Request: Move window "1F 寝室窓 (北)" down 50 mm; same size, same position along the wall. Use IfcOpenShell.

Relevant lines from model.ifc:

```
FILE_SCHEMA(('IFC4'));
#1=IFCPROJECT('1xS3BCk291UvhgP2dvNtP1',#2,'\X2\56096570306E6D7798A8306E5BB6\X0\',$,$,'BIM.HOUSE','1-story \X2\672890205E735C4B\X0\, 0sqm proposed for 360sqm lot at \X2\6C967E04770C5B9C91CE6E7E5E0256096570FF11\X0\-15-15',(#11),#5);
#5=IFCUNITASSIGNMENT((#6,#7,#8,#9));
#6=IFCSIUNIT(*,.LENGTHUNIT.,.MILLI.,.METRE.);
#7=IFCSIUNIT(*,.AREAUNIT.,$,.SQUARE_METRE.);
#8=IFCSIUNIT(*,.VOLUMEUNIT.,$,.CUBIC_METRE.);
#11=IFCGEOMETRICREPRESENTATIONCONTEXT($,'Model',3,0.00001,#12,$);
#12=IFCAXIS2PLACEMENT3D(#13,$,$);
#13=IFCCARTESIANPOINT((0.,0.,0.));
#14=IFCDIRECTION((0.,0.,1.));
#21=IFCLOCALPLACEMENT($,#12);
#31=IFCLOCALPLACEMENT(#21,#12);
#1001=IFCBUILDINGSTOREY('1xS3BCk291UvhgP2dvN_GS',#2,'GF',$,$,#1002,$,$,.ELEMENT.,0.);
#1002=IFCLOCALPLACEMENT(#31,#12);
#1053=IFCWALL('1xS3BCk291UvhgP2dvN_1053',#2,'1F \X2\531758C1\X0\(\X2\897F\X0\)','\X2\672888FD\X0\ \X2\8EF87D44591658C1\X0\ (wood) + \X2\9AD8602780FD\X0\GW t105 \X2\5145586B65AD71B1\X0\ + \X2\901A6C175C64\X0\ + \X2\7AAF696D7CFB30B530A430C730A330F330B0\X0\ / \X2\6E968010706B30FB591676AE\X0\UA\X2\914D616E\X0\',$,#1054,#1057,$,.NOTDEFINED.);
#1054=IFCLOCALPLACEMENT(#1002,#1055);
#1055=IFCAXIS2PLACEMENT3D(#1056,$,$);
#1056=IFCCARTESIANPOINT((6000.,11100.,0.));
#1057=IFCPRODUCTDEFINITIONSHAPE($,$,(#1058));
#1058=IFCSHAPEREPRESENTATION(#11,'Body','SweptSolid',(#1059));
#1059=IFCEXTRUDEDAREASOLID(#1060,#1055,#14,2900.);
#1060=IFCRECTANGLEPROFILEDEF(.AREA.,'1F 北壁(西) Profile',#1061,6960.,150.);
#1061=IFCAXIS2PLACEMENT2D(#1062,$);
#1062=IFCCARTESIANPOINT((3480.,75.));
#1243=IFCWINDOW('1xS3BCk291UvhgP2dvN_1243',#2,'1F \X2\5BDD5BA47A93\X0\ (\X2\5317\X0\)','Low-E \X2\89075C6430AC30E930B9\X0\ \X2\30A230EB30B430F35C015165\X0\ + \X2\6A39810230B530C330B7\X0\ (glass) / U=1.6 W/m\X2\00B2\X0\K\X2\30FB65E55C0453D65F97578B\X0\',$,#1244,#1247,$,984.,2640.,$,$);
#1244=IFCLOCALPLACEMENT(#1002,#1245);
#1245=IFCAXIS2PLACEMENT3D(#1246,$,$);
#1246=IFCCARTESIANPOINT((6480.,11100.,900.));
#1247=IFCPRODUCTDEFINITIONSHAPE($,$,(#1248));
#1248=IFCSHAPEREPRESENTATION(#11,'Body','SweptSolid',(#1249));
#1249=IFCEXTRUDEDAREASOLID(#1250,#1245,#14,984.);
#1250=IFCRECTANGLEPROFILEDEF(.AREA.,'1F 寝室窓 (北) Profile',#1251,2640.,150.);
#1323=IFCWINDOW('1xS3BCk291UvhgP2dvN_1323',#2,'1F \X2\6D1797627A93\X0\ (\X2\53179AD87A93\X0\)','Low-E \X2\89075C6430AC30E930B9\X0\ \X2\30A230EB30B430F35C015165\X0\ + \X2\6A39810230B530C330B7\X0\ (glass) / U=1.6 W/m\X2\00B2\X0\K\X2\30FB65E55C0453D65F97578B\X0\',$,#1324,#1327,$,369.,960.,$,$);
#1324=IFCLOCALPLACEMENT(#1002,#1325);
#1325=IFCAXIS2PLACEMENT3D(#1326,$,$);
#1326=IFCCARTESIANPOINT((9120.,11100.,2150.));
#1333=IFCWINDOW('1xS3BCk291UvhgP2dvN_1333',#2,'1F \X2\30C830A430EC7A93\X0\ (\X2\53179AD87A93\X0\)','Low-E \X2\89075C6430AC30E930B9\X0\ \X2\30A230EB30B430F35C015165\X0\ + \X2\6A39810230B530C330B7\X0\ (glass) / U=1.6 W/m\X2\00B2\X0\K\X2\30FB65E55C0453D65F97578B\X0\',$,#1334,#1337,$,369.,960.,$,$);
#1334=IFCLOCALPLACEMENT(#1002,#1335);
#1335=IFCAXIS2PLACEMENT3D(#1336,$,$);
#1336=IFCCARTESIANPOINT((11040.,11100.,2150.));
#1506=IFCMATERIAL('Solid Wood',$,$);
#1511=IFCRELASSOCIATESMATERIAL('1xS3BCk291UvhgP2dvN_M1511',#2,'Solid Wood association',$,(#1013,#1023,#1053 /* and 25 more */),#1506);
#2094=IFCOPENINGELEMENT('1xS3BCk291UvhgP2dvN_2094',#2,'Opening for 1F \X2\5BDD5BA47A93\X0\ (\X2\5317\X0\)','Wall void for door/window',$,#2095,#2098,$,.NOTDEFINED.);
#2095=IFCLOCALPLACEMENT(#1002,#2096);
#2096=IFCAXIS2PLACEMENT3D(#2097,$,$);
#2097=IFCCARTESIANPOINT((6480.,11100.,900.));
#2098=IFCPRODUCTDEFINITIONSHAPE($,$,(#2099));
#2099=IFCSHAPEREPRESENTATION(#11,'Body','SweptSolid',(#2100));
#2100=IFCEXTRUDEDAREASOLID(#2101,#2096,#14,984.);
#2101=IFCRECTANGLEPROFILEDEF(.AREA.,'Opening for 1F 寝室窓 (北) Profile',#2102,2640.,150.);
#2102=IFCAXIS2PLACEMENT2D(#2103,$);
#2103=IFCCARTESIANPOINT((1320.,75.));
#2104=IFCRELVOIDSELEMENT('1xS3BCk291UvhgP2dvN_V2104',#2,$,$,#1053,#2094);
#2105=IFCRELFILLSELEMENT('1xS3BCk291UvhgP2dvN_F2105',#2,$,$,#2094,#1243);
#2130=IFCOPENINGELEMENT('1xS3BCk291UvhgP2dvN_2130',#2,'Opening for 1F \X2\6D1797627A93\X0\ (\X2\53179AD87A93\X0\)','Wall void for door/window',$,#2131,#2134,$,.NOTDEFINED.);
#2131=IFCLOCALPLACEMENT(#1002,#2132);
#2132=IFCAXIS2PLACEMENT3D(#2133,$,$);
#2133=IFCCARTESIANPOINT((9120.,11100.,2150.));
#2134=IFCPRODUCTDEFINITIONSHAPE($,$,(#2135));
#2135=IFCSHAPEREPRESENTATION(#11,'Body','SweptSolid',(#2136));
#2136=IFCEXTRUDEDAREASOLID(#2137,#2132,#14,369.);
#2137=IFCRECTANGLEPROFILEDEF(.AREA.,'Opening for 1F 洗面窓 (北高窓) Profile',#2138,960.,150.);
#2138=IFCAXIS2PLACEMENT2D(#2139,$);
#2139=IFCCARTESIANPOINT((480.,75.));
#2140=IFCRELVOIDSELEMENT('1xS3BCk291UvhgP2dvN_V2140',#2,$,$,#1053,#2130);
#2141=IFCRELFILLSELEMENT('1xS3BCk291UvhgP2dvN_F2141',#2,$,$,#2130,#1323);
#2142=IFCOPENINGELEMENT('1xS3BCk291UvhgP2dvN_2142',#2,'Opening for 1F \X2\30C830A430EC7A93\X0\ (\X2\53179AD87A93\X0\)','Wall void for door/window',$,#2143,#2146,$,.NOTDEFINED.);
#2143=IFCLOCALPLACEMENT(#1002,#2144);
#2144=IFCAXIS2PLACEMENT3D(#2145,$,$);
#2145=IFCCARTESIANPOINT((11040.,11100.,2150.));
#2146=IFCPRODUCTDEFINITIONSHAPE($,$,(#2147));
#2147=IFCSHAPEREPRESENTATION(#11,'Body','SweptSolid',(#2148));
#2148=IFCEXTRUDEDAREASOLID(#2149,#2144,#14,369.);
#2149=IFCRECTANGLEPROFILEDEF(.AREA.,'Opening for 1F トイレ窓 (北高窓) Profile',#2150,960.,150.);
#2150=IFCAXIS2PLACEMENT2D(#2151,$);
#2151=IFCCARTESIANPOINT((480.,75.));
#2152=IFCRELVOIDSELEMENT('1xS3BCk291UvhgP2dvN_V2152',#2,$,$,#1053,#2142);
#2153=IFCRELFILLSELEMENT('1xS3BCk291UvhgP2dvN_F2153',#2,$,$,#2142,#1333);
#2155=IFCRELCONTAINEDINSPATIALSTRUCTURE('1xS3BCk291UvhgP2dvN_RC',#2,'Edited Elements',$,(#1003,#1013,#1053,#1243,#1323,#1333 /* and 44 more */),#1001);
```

```python
import numpy as np
import ifcopenshell
import ifcopenshell.api.geometry
import ifcopenshell.util.placement
import ifcopenshell.util.unit

model = ifcopenshell.open("model.ifc")
unit_scale = ifcopenshell.util.unit.calculate_unit_scale(model)

window = model.by_guid("1xS3BCk291UvhgP2dvN_1243")
opening = window.FillsVoids[0].RelatingOpeningElement
dz = -0.05 / unit_scale

shift = np.array([0.0, 0.0, dz])
# The window is not placed relative to its opening, so move both.
for product in (opening, window):
    matrix = ifcopenshell.util.placement.get_local_placement(product.ObjectPlacement)
    matrix[:3, 3] += shift
    ifcopenshell.api.geometry.edit_object_placement(model, product=product, matrix=matrix, is_si=False)

print(f"moved by {dz * unit_scale:+.3f} m")

model.write("model_edited.ifc")
```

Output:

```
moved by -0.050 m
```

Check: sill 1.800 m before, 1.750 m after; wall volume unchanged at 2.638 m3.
